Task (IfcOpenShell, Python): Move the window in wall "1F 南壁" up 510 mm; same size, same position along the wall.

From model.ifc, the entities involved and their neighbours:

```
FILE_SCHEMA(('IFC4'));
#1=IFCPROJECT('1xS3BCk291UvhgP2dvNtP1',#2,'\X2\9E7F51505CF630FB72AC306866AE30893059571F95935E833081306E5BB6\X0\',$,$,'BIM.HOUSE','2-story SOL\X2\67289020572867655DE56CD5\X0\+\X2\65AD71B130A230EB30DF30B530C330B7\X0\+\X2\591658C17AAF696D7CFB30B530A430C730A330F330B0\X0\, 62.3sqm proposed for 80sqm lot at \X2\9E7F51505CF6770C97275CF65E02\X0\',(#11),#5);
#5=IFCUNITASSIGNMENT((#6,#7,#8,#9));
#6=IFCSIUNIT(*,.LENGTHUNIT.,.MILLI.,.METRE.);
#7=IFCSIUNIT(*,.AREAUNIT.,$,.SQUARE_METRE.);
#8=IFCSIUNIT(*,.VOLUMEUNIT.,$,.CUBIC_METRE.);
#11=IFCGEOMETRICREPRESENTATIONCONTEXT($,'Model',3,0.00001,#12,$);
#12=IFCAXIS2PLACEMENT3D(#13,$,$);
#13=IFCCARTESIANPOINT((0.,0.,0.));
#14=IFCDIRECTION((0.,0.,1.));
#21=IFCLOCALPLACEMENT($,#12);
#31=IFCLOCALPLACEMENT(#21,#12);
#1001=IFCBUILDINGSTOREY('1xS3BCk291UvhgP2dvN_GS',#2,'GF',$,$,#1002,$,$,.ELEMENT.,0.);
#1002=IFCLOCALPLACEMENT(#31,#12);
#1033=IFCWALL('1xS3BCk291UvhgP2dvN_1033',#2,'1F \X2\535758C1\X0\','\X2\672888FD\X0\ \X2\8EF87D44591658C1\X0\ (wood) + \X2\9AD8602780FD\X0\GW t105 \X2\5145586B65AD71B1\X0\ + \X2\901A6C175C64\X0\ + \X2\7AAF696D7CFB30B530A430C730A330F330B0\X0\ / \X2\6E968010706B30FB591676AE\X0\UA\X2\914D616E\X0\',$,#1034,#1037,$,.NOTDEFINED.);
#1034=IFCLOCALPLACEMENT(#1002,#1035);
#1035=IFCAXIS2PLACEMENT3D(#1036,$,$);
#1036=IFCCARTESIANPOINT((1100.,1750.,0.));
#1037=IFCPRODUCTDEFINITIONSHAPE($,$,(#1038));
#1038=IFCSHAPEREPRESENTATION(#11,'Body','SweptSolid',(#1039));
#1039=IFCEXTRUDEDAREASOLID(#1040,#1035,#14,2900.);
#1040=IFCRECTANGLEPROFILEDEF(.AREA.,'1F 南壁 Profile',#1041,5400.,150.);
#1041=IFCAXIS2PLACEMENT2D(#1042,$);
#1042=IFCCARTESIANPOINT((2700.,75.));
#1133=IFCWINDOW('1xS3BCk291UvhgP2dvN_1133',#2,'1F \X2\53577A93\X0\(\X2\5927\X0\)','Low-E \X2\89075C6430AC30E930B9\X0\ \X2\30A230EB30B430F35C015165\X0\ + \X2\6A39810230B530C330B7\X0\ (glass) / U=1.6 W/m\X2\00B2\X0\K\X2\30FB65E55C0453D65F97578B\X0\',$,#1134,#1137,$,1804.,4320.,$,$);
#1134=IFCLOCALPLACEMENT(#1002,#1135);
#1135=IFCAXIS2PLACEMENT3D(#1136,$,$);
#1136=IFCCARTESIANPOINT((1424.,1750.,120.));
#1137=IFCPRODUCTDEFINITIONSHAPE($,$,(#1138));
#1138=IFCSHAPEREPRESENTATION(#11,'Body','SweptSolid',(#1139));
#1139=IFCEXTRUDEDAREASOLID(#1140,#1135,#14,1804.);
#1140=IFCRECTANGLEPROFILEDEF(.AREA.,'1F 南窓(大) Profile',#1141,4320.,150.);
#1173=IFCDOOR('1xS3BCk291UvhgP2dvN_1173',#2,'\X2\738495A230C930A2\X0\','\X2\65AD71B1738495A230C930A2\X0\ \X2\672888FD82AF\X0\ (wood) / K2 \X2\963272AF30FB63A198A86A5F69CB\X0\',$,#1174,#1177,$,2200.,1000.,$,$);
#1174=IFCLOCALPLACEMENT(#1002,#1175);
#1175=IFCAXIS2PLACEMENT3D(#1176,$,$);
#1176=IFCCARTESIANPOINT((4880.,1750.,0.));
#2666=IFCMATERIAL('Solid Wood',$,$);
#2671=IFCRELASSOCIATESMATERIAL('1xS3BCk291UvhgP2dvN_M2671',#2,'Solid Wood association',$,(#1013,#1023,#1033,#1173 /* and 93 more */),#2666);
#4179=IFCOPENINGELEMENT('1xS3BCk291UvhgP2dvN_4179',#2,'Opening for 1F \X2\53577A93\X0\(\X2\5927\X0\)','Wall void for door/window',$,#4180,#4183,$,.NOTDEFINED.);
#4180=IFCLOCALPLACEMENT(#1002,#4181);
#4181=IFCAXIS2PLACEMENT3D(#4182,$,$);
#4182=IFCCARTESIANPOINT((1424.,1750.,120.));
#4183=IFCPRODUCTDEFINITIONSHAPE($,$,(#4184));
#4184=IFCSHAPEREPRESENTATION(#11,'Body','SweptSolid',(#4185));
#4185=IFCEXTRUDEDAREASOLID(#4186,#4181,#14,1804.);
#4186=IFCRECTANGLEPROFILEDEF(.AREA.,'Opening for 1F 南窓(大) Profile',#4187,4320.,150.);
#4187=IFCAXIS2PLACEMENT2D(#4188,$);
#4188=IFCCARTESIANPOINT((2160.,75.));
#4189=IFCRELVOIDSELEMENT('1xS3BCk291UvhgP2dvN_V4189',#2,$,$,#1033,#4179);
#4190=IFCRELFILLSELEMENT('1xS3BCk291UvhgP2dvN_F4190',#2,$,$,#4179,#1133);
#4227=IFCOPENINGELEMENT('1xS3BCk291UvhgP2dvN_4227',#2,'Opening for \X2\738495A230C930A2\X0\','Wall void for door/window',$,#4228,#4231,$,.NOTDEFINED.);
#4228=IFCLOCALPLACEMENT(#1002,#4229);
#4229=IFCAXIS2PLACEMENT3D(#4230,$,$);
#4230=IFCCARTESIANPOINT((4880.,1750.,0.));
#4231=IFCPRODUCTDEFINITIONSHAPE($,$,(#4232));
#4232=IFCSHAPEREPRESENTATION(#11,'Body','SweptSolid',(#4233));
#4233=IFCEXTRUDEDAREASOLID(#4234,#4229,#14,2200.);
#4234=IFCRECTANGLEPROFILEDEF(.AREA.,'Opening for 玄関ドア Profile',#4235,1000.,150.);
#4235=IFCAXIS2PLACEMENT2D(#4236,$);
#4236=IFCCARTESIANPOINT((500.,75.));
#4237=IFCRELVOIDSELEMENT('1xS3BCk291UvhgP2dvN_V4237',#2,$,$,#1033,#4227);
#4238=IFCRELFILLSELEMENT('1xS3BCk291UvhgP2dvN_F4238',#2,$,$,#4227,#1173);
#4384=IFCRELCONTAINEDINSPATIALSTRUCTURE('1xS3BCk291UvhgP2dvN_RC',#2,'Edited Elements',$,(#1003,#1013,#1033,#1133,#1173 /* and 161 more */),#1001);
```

```python
import numpy as np
import ifcopenshell
import ifcopenshell.api.geometry
import ifcopenshell.util.placement
import ifcopenshell.util.unit

model = ifcopenshell.open("model.ifc")
unit_scale = ifcopenshell.util.unit.calculate_unit_scale(model)

window = model.by_guid("1xS3BCk291UvhgP2dvN_1133")
opening = window.FillsVoids[0].RelatingOpeningElement
dz = 0.51 / unit_scale

shift = np.array([0.0, 0.0, dz])
# The window is not placed relative to its opening, so move both.
for product in (opening, window):
    matrix = ifcopenshell.util.placement.get_local_placement(product.ObjectPlacement)
    matrix[:3, 3] += shift
    ifcopenshell.api.geometry.edit_object_placement(model, product=product, matrix=matrix, is_si=False)

print(f"moved by {dz * unit_scale:+.3f} m")

model.write("model_v2.ifc")
```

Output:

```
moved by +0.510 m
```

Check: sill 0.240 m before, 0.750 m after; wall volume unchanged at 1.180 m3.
